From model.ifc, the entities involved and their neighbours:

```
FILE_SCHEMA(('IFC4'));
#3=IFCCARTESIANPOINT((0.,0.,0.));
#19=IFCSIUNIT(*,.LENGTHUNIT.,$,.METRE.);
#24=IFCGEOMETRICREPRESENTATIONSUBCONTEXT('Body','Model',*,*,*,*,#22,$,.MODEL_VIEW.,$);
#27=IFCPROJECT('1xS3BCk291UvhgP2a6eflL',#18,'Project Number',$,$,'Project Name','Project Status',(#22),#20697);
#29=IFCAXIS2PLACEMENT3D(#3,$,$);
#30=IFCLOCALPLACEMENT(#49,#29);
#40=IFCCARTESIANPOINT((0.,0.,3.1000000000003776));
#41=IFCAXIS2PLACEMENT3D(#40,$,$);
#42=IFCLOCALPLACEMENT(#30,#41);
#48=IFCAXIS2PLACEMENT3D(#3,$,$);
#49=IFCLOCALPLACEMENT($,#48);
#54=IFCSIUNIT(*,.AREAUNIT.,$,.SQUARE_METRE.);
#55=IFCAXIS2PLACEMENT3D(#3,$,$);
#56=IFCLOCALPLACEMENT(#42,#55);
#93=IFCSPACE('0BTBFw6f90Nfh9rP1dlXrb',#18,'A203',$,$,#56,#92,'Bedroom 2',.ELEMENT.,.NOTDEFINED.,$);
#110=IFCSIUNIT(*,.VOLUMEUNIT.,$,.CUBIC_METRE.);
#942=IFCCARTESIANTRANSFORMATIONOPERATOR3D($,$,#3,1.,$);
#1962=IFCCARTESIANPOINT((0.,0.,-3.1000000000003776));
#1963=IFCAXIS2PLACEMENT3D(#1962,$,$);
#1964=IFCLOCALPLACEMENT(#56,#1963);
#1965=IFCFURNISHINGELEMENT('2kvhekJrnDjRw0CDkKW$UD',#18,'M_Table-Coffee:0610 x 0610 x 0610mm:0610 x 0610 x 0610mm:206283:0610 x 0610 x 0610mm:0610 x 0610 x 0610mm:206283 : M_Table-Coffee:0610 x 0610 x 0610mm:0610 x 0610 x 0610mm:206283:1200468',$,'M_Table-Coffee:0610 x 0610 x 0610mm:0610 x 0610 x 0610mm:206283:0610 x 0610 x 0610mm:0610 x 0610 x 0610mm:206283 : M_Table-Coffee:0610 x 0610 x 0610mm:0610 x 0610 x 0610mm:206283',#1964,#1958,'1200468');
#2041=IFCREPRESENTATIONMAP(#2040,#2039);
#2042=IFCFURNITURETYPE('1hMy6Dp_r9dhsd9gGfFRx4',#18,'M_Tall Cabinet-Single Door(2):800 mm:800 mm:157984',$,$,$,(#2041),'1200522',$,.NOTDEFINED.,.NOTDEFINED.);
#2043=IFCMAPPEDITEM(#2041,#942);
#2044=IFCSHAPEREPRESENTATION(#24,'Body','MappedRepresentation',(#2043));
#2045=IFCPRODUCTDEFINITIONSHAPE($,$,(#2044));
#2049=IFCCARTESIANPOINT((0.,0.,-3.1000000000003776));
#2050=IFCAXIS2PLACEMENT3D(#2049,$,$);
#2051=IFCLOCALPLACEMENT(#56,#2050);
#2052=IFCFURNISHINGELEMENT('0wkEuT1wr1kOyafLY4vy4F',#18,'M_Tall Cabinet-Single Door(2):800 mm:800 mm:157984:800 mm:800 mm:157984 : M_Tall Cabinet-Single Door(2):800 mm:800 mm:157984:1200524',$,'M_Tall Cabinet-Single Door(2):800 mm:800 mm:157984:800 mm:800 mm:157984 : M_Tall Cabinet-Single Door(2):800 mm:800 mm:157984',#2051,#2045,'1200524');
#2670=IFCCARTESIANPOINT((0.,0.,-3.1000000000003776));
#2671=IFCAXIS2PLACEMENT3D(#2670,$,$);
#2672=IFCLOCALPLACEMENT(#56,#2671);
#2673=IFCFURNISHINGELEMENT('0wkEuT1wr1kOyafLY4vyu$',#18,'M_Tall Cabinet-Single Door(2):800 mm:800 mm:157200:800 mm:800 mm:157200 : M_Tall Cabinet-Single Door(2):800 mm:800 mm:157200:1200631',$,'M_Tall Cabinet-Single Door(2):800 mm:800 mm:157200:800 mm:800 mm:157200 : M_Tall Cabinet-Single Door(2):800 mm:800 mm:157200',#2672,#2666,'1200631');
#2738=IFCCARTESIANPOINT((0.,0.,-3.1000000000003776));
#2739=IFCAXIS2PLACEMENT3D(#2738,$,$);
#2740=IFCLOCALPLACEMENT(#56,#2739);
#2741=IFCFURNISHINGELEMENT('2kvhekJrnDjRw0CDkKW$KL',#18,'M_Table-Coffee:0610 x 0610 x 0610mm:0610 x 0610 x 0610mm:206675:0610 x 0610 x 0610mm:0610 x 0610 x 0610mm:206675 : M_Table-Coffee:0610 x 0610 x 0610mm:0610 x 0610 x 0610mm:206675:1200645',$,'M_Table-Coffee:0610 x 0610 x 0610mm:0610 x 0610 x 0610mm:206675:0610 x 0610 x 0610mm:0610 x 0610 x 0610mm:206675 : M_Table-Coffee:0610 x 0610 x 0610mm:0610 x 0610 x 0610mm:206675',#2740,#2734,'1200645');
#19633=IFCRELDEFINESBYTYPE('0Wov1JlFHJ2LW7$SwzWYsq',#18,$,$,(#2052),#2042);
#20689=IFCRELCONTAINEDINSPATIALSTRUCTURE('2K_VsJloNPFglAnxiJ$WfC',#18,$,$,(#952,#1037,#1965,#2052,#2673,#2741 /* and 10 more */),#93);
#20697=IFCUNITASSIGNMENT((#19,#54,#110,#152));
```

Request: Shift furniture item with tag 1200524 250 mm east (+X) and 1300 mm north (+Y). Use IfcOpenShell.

```python
import ifcopenshell
import ifcopenshell.api.geometry
import ifcopenshell.util.placement

model = ifcopenshell.open("model.ifc")

item = model.by_id(2052)
matrix = ifcopenshell.util.placement.get_local_placement(item.ObjectPlacement)
matrix[0, 3] += 0.25
matrix[1, 3] += 1.3
ifcopenshell.api.geometry.edit_object_placement(model, product=item, matrix=matrix, is_si=False)

print(ifcopenshell.util.placement.get_local_placement(item.ObjectPlacement).round(3) + 0.0)

model.write("model_updated.ifc")
```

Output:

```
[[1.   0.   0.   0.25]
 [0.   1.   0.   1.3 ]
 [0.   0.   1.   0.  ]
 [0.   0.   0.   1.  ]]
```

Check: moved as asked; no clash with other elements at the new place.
